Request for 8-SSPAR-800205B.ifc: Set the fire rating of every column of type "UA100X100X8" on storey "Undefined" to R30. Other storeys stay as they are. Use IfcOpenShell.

First a look at what the model holds.

```python
import ifcopenshell
import ifcopenshell.util.element

model = ifcopenshell.open("8-SSPAR-800205B.ifc")
print(model.schema)
storey = next(s for s in model.by_type("IfcBuildingStorey") if s.Name == "Undefined")
columns = [e for e in ifcopenshell.util.element.get_decomposition(storey) if e.is_a("IfcColumn")]
seen = {}
for e in columns:
    element_type = ifcopenshell.util.element.get_type(e)
    key = (element_type.Name if element_type != e and element_type else None, ifcopenshell.util.element.get_pset(e, "Pset_ColumnCommon", "FireRating"))
    seen[key] = seen.get(key, 0) + 1
for (name, value), count in sorted(seen.items(), key=str):
    print(count, "x", name, "|", value)
```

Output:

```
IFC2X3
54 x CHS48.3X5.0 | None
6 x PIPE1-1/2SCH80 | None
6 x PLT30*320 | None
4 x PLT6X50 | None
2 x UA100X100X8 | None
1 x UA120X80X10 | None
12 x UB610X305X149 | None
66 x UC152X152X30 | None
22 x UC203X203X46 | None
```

```python
import ifcopenshell
import ifcopenshell.api.pset
import ifcopenshell.util.element

model = ifcopenshell.open("8-SSPAR-800205B.ifc")

storey = next(s for s in model.by_type("IfcBuildingStorey") if s.Name == "Undefined")
columns = [e for e in ifcopenshell.util.element.get_decomposition(storey) if e.is_a("IfcColumn")]

count = 0
for e in columns:
    element_type = ifcopenshell.util.element.get_type(e)
    if element_type in (None, e) or element_type.Name != "UA100X100X8":
        continue
    # add_pset returns the element's existing set when there is one.
    pset = ifcopenshell.api.pset.add_pset(model, product=e, name="Pset_ColumnCommon")
    ifcopenshell.api.pset.edit_pset(model, pset=pset, properties={"FireRating": "R30"})
    count += 1

print(count, "columns updated")

model.write("8-SSPAR-800205B_v2.ifc")
```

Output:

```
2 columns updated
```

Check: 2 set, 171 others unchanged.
